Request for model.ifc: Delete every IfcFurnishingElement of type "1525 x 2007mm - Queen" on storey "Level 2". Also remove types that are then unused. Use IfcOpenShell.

First a look at what the model holds.

```python
import ifcopenshell
import ifcopenshell.util.element

model = ifcopenshell.open("model.ifc")
print(model.schema)
storey = next(s for s in model.by_type("IfcBuildingStorey") if s.Name == "Level 2")
furniture = [e for e in ifcopenshell.util.element.get_decomposition(storey) if e.is_a("IfcFurnishingElement")]
seen = {}
for e in furniture:
    element_type = ifcopenshell.util.element.get_type(e)
    name = element_type.Name if element_type not in (None, e) else None
    seen[name] = seen.get(name, 0) + 1
for name, count in sorted(seen.items(), key=str):
    print(count, "x", name)
```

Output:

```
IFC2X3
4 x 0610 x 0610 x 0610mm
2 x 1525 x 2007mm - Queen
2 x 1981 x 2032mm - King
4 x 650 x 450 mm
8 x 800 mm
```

```python
import ifcopenshell
import ifcopenshell.api.root
import ifcopenshell.util.element

model = ifcopenshell.open("model.ifc")

storey = next(s for s in model.by_type("IfcBuildingStorey") if s.Name == "Level 2")
furniture = [e for e in ifcopenshell.util.element.get_decomposition(storey) if e.is_a("IfcFurnishingElement")]
targets = [e for e in furniture if (t := ifcopenshell.util.element.get_type(e)) not in (None, e) and t.Name == "1525 x 2007mm - Queen"]
types = {ifcopenshell.util.element.get_type(e) for e in targets} - {None, *targets}

for e in targets:
    ifcopenshell.api.root.remove_product(model, product=e)
print(len(targets), "removed")

unused = [t for t in types if not ifcopenshell.util.element.get_types(t)]
for t in unused:
    ifcopenshell.api.root.remove_product(model, product=t)
print(len(unused), "unused types removed")

model.write("model_edited.ifc")
```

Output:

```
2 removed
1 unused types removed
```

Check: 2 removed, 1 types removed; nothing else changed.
